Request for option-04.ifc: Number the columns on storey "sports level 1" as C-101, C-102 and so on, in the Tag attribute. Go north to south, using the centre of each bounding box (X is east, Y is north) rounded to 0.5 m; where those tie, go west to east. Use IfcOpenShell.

First a look at what the model holds.

```python
import ifcopenshell
import ifcopenshell.util.element
import ifcopenshell.util.placement

model = ifcopenshell.open("option-04.ifc")
print(model.schema)
storey = next(s for s in model.by_type("IfcBuildingStorey") if s.Name == "sports level 1")
columns = [e for e in ifcopenshell.util.element.get_decomposition(storey) if e.is_a("IfcColumn")]
for e in sorted(columns, key=lambda e: e.id()):
    origin = ifcopenshell.util.placement.get_local_placement(e.ObjectPlacement)[:3, 3]
    print(e.id(), e.Tag, e.Name, origin.round(2) + 0.0, sep=" | ")
```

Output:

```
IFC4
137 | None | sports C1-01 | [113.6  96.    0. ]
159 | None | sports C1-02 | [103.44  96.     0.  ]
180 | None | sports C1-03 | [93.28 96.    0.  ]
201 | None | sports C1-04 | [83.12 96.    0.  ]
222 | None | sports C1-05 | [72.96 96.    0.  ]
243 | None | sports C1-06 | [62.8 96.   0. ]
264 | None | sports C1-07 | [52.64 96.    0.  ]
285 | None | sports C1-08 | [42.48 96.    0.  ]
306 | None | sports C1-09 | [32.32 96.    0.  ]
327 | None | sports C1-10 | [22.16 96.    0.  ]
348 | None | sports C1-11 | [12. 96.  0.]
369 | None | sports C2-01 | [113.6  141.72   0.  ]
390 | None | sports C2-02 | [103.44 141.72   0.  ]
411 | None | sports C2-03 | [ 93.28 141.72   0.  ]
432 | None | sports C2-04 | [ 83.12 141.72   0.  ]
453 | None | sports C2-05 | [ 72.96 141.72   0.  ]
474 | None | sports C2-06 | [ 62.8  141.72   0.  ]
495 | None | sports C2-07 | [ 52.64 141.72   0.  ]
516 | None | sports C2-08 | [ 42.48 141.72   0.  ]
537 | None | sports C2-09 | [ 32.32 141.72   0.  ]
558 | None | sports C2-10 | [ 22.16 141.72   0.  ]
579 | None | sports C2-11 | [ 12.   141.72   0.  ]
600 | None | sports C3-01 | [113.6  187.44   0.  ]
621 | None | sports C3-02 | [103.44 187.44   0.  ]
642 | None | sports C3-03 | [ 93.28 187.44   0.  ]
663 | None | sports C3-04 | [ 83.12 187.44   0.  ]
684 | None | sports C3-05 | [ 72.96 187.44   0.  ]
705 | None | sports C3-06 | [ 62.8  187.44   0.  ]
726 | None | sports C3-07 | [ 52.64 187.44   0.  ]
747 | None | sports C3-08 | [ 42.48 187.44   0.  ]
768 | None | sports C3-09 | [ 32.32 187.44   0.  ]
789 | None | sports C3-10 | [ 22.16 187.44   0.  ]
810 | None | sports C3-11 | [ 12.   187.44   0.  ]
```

```python
import ifcopenshell
import ifcopenshell.geom
import ifcopenshell.util.element
import ifcopenshell.util.shape

model = ifcopenshell.open("option-04.ifc")
settings = ifcopenshell.geom.settings()
settings.set("use-world-coords", True)


def centre(element):
    shape = ifcopenshell.geom.create_shape(settings, element)
    return ifcopenshell.util.shape.get_bbox_centroid(shape.geometry)


storey = next(s for s in model.by_type("IfcBuildingStorey") if s.Name == "sports level 1")
columns = [e for e in ifcopenshell.util.element.get_decomposition(storey) if e.is_a("IfcColumn")]

# Insertion points can sit at a corner or the storey origin, so sort by the geometry (in metres).
centres = {e: centre(e) for e in columns}
columns.sort(key=lambda e: (-round(centres[e][1] / 0.5), centres[e][0]))

for i, e in enumerate(columns, start=1):
    number = f"C-1{i:02d}"
    e.Tag = number
    print(e.id(), number)

model.write("option-04_rev.ifc")
```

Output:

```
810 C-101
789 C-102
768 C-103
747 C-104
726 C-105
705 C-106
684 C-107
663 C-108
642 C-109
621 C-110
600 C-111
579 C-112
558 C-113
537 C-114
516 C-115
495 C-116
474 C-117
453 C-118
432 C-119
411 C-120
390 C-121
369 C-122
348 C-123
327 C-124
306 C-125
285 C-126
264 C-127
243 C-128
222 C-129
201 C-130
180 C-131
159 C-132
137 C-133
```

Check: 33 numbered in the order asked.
